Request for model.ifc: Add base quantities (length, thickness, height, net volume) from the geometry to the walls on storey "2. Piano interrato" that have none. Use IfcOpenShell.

First a look at what the model holds.

```python
import ifcopenshell
import ifcopenshell.util.element
import ifcopenshell.util.unit

model = ifcopenshell.open("model.ifc")
print(model.schema)
for unit_type in ("LENGTHUNIT", "AREAUNIT", "VOLUMEUNIT"):
    print(unit_type, ifcopenshell.util.unit.calculate_unit_scale(model, unit_type))
storey = next(s for s in model.by_type("IfcBuildingStorey") if s.Name == "2. Piano interrato")
walls = [e for e in ifcopenshell.util.element.get_decomposition(storey) if e.is_a("IfcWall")]
for e in sorted(walls, key=lambda e: e.id()):
    print(e.id(), e.is_a(), e.Name, list(ifcopenshell.util.element.get_psets(e, qtos_only=True)), sep=" | ")
```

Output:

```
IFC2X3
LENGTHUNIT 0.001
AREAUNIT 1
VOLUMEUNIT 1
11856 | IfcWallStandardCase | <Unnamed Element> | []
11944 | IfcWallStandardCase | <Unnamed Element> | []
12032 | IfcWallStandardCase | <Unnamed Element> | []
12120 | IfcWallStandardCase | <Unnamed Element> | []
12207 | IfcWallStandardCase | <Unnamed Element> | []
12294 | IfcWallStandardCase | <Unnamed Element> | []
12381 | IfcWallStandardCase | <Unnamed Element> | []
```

```python
import ifcopenshell
import ifcopenshell.api.pset
import ifcopenshell.geom
import ifcopenshell.util.element
import ifcopenshell.util.shape
import ifcopenshell.util.unit

model = ifcopenshell.open("model.ifc")
unit_scale = ifcopenshell.util.unit.calculate_unit_scale(model)
volume_scale = ifcopenshell.util.unit.calculate_unit_scale(model, "VOLUMEUNIT")
settings = ifcopenshell.geom.settings()

storey = next(s for s in model.by_type("IfcBuildingStorey") if s.Name == "2. Piano interrato")
walls = [e for e in ifcopenshell.util.element.get_decomposition(storey) if e.is_a("IfcWall")]

for e in sorted(walls, key=lambda e: e.id()):
    if ifcopenshell.util.element.get_psets(e, qtos_only=True, should_inherit=False):
        continue
    # Geometry comes back in metres, in the element's own axes.
    shape = ifcopenshell.geom.create_shape(settings, e)
    values = {
        "Length": ifcopenshell.util.shape.get_x(shape.geometry) / unit_scale,
        "Width": ifcopenshell.util.shape.get_y(shape.geometry) / unit_scale,
        "Height": ifcopenshell.util.shape.get_z(shape.geometry) / unit_scale,
        "NetVolume": ifcopenshell.util.shape.get_volume(shape.geometry) / volume_scale,
    }
    qto = ifcopenshell.api.pset.add_qto(model, product=e, name="BaseQuantities")
    ifcopenshell.api.pset.edit_qto(model, qto=qto, properties=values)
    print(e.id(), {k: round(v, 3) for k, v in values.items()})

model.write("model_edited.ifc")
```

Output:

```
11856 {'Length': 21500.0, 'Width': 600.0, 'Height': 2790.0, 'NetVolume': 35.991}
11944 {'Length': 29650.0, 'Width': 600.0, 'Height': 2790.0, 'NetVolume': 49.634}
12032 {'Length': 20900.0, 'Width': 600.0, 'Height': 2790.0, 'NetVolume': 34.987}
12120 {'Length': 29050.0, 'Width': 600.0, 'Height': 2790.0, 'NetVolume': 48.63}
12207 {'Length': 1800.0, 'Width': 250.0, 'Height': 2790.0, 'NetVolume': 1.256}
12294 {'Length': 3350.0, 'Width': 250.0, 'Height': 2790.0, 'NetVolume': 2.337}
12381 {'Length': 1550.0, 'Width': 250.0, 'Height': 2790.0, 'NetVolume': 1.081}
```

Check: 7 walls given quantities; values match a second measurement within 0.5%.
